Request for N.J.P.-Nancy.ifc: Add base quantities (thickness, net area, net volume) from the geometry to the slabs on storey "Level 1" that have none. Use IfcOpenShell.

First a look at what the model holds.

```python
import ifcopenshell
import ifcopenshell.util.element
import ifcopenshell.util.unit

model = ifcopenshell.open("N.J.P.-Nancy.ifc")
print(model.schema)
for unit_type in ("LENGTHUNIT", "AREAUNIT", "VOLUMEUNIT"):
    print(unit_type, ifcopenshell.util.unit.calculate_unit_scale(model, unit_type))
storey = next(s for s in model.by_type("IfcBuildingStorey") if s.Name == "Level 1")
slabs = [e for e in ifcopenshell.util.element.get_decomposition(storey) if e.is_a("IfcSlab")]
for e in sorted(slabs, key=lambda e: e.id()):
    print(e.id(), e.is_a(), e.Name, list(ifcopenshell.util.element.get_psets(e, qtos_only=True)), sep=" | ")
```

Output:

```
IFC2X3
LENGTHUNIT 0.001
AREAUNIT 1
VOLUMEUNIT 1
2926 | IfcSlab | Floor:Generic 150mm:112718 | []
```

```python
import ifcopenshell
import ifcopenshell.api.pset
import ifcopenshell.geom
import ifcopenshell.util.element
import ifcopenshell.util.shape
import ifcopenshell.util.unit

model = ifcopenshell.open("N.J.P.-Nancy.ifc")
unit_scale = ifcopenshell.util.unit.calculate_unit_scale(model)
area_scale = ifcopenshell.util.unit.calculate_unit_scale(model, "AREAUNIT")
volume_scale = ifcopenshell.util.unit.calculate_unit_scale(model, "VOLUMEUNIT")
settings = ifcopenshell.geom.settings()

storey = next(s for s in model.by_type("IfcBuildingStorey") if s.Name == "Level 1")
slabs = [e for e in ifcopenshell.util.element.get_decomposition(storey) if e.is_a("IfcSlab")]

for e in sorted(slabs, key=lambda e: e.id()):
    if ifcopenshell.util.element.get_psets(e, qtos_only=True, should_inherit=False):
        continue
    # Geometry comes back in metres, in the element's own axes.
    shape = ifcopenshell.geom.create_shape(settings, e)
    values = {
        "Width": ifcopenshell.util.shape.get_z(shape.geometry) / unit_scale,
        "NetArea": ifcopenshell.util.shape.get_footprint_area(shape.geometry) / area_scale,
        "NetVolume": ifcopenshell.util.shape.get_volume(shape.geometry) / volume_scale,
    }
    qto = ifcopenshell.api.pset.add_qto(model, product=e, name="BaseQuantities")
    ifcopenshell.api.pset.edit_qto(model, qto=qto, properties=values)
    print(e.id(), {k: round(v, 3) for k, v in values.items()})

model.write("N.J.P.-Nancy_v2.ifc")
```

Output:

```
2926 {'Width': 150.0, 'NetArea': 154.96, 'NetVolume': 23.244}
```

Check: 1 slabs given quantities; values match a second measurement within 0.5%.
